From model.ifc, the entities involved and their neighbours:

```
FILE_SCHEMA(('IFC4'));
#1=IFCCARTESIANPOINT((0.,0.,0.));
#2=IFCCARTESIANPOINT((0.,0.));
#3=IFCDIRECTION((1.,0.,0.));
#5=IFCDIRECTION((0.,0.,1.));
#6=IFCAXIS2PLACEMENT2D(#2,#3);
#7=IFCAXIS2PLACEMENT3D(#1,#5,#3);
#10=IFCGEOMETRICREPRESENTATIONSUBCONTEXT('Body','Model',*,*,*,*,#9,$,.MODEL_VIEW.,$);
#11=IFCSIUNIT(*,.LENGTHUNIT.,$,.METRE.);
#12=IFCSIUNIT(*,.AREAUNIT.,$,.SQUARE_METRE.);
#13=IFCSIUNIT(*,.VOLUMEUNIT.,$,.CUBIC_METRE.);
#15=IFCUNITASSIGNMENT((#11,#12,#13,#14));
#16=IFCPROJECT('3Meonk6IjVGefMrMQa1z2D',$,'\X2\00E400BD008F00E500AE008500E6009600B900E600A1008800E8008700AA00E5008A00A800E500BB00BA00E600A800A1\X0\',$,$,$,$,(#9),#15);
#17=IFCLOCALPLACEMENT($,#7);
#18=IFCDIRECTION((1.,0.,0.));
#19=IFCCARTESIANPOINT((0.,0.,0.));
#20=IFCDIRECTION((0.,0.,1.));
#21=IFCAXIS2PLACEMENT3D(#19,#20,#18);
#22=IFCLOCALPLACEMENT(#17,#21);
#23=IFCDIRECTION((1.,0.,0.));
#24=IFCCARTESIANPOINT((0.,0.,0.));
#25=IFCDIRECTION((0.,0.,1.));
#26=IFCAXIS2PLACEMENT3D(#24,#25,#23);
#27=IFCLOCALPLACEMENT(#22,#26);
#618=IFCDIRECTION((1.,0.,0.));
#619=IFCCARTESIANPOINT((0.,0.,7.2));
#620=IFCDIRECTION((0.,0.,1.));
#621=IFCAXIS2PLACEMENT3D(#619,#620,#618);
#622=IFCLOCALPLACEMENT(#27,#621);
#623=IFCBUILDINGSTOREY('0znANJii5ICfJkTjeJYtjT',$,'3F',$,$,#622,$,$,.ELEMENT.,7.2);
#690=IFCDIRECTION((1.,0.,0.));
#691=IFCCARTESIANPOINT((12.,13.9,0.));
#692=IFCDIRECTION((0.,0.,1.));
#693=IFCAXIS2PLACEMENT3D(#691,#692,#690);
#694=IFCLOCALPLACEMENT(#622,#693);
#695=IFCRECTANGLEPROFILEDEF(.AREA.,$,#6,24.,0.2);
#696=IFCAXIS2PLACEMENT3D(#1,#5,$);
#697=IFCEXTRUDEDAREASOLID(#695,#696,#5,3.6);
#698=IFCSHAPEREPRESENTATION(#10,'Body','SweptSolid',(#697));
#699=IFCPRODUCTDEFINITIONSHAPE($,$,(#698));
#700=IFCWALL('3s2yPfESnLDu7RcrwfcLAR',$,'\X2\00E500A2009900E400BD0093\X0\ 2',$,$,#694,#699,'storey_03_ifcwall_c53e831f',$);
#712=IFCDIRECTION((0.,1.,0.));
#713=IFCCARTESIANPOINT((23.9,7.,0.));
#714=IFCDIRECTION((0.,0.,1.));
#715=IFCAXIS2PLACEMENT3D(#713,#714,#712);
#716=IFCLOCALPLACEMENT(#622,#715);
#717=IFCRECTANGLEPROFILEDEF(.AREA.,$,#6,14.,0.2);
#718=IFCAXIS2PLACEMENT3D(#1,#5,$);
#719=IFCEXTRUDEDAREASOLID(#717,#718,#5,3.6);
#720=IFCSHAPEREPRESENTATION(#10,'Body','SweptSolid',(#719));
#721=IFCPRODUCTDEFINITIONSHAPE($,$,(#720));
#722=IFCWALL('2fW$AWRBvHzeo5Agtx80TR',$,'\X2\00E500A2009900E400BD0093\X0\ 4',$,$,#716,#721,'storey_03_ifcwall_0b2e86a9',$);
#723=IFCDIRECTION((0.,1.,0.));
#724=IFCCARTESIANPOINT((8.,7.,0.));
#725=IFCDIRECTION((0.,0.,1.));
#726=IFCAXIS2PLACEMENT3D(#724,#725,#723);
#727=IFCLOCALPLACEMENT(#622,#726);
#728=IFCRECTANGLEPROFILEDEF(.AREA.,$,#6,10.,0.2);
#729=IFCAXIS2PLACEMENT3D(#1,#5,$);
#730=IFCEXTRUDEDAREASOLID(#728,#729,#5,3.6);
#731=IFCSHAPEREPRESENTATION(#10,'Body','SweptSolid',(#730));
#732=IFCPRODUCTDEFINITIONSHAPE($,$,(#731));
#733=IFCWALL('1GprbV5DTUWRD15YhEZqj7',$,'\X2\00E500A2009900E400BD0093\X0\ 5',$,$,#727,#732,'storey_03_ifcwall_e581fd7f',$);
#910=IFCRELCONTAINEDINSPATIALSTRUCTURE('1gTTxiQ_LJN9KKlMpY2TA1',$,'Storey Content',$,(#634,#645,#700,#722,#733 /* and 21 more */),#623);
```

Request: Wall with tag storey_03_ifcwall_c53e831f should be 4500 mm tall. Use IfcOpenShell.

```python
import ifcopenshell
import ifcopenshell.geom
import ifcopenshell.util.representation
import ifcopenshell.util.shape
import ifcopenshell.util.unit

model = ifcopenshell.open("model.ifc")
unit_scale = ifcopenshell.util.unit.calculate_unit_scale(model)
settings = ifcopenshell.geom.settings()


def volume(element):
    """Net volume in cubic metres, openings subtracted."""
    shape = ifcopenshell.geom.create_shape(settings, element)
    return ifcopenshell.util.shape.get_volume(shape.geometry)


wall = model.by_guid("3s2yPfESnLDu7RcrwfcLAR")
before = volume(wall)

body = ifcopenshell.util.representation.get_representation(wall, "Model", "Body")
solid = body.Items[0]
old_height = solid.Depth
solid.Depth = 4.5 / unit_scale
after = volume(wall)

print(f"height {old_height:g} -> {solid.Depth:g}, volume {before:.3f} -> {after:.3f} m3")

model.write("model_rev.ifc")
```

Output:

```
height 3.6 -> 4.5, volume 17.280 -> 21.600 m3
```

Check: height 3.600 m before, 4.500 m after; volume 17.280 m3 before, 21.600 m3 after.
